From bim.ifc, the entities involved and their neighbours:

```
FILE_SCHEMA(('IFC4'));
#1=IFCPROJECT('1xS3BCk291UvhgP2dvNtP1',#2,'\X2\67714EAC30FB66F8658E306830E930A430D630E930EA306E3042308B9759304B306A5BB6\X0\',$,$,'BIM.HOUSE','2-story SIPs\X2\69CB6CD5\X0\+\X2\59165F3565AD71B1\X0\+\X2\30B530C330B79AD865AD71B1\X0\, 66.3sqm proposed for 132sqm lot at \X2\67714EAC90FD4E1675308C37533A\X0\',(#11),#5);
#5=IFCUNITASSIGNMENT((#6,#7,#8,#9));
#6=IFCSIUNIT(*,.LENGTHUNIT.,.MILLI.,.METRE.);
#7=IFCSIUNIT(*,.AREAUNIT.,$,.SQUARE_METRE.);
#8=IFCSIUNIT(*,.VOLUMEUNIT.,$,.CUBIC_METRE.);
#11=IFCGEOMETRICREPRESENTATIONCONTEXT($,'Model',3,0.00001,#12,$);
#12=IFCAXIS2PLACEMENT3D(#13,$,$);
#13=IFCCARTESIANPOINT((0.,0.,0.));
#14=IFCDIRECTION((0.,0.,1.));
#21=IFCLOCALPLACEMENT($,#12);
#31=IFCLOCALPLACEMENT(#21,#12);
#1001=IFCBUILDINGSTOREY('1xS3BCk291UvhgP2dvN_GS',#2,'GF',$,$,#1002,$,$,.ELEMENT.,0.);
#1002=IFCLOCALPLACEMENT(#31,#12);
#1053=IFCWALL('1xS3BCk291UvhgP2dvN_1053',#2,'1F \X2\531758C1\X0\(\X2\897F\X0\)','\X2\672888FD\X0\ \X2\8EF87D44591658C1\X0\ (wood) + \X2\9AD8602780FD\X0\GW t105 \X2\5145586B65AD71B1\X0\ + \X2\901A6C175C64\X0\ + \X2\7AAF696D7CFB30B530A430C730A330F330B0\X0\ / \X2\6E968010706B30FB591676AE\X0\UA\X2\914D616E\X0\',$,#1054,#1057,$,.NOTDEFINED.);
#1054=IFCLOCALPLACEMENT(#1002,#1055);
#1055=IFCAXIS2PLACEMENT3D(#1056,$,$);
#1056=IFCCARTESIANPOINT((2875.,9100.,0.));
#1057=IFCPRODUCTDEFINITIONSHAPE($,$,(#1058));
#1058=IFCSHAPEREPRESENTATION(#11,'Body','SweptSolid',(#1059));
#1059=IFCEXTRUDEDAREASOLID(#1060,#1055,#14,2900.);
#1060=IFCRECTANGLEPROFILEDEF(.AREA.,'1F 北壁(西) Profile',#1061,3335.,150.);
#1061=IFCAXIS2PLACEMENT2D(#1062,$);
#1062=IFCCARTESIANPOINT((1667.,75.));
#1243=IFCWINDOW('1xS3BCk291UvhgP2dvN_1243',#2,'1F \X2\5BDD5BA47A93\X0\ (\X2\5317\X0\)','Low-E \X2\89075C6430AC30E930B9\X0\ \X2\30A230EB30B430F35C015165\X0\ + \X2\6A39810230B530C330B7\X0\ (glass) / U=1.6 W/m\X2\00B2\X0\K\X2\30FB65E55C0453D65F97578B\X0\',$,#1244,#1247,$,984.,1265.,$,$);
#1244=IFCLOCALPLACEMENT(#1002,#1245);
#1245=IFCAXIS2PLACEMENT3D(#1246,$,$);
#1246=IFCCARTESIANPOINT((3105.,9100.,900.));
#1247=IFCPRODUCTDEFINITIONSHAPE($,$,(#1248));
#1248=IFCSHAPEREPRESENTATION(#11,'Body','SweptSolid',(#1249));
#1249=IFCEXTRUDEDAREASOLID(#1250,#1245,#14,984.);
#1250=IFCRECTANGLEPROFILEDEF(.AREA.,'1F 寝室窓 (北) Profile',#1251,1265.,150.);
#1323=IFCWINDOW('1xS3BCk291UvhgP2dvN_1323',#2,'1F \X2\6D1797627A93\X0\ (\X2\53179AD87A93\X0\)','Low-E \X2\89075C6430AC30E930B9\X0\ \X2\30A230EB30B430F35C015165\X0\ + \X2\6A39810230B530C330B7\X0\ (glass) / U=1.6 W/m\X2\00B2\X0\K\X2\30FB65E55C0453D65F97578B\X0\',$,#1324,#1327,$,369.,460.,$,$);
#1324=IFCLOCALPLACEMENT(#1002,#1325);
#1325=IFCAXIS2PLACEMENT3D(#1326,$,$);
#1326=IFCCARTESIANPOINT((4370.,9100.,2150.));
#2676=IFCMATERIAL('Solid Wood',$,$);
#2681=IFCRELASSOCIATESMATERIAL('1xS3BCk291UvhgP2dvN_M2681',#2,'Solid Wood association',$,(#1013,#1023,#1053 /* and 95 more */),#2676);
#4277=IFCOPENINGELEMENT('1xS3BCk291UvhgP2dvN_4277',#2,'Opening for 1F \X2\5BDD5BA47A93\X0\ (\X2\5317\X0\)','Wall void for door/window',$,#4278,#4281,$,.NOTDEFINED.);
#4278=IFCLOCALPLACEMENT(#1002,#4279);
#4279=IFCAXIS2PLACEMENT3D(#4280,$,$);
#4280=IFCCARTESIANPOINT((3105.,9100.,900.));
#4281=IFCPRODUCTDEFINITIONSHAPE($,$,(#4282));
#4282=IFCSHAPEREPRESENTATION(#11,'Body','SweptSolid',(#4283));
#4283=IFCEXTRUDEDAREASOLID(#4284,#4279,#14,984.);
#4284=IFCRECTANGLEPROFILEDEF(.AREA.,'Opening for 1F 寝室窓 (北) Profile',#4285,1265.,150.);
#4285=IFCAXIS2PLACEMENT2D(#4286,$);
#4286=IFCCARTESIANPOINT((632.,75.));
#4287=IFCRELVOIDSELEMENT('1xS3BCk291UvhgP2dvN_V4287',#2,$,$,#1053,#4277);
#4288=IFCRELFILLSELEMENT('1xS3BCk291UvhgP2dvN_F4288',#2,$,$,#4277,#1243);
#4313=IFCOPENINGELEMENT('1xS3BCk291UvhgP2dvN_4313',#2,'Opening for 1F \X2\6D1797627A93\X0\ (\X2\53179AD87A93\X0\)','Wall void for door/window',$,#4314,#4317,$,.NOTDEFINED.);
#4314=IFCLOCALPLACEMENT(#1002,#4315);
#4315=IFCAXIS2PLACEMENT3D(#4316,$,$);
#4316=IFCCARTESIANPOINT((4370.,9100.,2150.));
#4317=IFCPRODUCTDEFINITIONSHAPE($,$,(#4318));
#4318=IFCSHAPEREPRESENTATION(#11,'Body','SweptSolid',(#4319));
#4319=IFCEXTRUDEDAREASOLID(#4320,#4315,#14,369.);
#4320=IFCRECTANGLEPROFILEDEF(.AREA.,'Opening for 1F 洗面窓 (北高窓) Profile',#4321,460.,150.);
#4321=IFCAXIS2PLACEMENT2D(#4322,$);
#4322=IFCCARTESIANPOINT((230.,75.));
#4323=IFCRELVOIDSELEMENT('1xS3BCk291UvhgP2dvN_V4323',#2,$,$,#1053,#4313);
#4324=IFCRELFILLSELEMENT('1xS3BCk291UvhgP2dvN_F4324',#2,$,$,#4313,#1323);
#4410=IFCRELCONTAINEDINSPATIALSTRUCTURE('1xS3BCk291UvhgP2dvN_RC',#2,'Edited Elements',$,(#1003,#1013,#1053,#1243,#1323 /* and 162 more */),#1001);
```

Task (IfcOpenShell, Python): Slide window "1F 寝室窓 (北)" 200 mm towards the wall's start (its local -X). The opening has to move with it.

```python
import ifcopenshell
import ifcopenshell.api.geometry
import ifcopenshell.util.placement
import ifcopenshell.util.unit

model = ifcopenshell.open("bim.ifc")
unit_scale = ifcopenshell.util.unit.calculate_unit_scale(model)

window = model.by_guid("1xS3BCk291UvhgP2dvN_1243")
opening = window.FillsVoids[0].RelatingOpeningElement
wall = opening.VoidsElements[0].RelatingBuildingElement

wall_matrix = ifcopenshell.util.placement.get_local_placement(wall.ObjectPlacement)
shift = wall_matrix[:3, 0] * -0.2 / unit_scale
before = ifcopenshell.util.placement.get_local_placement(window.ObjectPlacement)[:3, 3].copy()

# The window is not placed relative to its opening, so move both.
for product in (opening, window):
    matrix = ifcopenshell.util.placement.get_local_placement(product.ObjectPlacement)
    matrix[:3, 3] += shift
    ifcopenshell.api.geometry.edit_object_placement(model, product=product, matrix=matrix, is_si=False)

after = ifcopenshell.util.placement.get_local_placement(window.ObjectPlacement)[:3, 3]
print("window moved by", (after - before).round(3) + 0.0)

model.write("bim_rev.ifc")
```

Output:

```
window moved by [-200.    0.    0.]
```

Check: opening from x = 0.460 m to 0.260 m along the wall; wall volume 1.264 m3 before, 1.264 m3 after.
